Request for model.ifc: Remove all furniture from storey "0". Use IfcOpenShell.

First a look at what the model holds.

```python
import ifcopenshell
import ifcopenshell.util.element

model = ifcopenshell.open("model.ifc")
print(model.schema)
storey = next(s for s in model.by_type("IfcBuildingStorey") if s.Name == "0")
furniture = [e for e in ifcopenshell.util.element.get_decomposition(storey) if e.is_a("IfcFurnishingElement")]
seen = {}
for e in furniture:
    element_type = ifcopenshell.util.element.get_type(e)
    name = element_type.Name if element_type not in (None, e) else None
    seen[name] = seen.get(name, 0) + 1
for name, count in sorted(seen.items(), key=str):
    print(count, "x", name)
```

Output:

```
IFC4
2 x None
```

```python
import ifcopenshell
import ifcopenshell.api.root
import ifcopenshell.util.element

model = ifcopenshell.open("model.ifc")

storey = next(s for s in model.by_type("IfcBuildingStorey") if s.Name == "0")
furniture = [e for e in ifcopenshell.util.element.get_decomposition(storey) if e.is_a("IfcFurnishingElement")]

for e in furniture:
    ifcopenshell.api.root.remove_product(model, product=e)
print(len(furniture), "removed")

model.write("model_updated.ifc")
```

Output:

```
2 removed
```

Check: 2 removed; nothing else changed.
